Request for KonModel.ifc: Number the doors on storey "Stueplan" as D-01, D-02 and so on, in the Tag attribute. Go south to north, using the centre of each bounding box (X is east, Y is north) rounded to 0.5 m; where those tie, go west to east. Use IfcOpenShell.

First a look at what the model holds.

```python
import ifcopenshell
import ifcopenshell.util.element
import ifcopenshell.util.placement

model = ifcopenshell.open("KonModel.ifc")
print(model.schema)
storey = next(s for s in model.by_type("IfcBuildingStorey") if s.Name == "Stueplan")
doors = [e for e in ifcopenshell.util.element.get_decomposition(storey) if e.is_a("IfcDoor")]
for e in sorted(doors, key=lambda e: e.id()):
    origin = ifcopenshell.util.placement.get_local_placement(e.ObjectPlacement)[:3, 3]
    print(e.id(), e.Tag, e.Name, origin.round(2) + 0.0, sep=" | ")
```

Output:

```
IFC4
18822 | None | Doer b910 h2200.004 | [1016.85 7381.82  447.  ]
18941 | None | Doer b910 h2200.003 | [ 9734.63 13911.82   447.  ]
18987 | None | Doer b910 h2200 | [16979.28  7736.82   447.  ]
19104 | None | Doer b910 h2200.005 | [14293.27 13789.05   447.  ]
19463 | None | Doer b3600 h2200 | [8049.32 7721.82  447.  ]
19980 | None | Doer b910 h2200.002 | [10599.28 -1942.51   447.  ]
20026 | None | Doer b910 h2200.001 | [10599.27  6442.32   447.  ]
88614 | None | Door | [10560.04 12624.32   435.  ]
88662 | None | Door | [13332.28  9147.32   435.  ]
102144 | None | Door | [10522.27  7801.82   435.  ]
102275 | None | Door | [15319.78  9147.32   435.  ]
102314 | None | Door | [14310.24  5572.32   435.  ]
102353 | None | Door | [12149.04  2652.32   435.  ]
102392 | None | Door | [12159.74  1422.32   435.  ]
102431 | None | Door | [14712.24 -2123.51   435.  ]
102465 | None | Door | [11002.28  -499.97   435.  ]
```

```python
import ifcopenshell
import ifcopenshell.geom
import ifcopenshell.util.element
import ifcopenshell.util.shape

model = ifcopenshell.open("KonModel.ifc")
settings = ifcopenshell.geom.settings()
settings.set("use-world-coords", True)


def centre(element):
    shape = ifcopenshell.geom.create_shape(settings, element)
    return ifcopenshell.util.shape.get_bbox_centroid(shape.geometry)


storey = next(s for s in model.by_type("IfcBuildingStorey") if s.Name == "Stueplan")
doors = [e for e in ifcopenshell.util.element.get_decomposition(storey) if e.is_a("IfcDoor")]

# Insertion points can sit at a corner or the storey origin, so sort by the geometry (in metres).
centres = {e: centre(e) for e in doors}
doors.sort(key=lambda e: (round(centres[e][1] / 0.5), centres[e][0]))

for i, e in enumerate(doors, start=1):
    number = f"D-{i:02d}"
    e.Tag = number
    print(e.id(), number)

model.write("KonModel_updated.ifc")
```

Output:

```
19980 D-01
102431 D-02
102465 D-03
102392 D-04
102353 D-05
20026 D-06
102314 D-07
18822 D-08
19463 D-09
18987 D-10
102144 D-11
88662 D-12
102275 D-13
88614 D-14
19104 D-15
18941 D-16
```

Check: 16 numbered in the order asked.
